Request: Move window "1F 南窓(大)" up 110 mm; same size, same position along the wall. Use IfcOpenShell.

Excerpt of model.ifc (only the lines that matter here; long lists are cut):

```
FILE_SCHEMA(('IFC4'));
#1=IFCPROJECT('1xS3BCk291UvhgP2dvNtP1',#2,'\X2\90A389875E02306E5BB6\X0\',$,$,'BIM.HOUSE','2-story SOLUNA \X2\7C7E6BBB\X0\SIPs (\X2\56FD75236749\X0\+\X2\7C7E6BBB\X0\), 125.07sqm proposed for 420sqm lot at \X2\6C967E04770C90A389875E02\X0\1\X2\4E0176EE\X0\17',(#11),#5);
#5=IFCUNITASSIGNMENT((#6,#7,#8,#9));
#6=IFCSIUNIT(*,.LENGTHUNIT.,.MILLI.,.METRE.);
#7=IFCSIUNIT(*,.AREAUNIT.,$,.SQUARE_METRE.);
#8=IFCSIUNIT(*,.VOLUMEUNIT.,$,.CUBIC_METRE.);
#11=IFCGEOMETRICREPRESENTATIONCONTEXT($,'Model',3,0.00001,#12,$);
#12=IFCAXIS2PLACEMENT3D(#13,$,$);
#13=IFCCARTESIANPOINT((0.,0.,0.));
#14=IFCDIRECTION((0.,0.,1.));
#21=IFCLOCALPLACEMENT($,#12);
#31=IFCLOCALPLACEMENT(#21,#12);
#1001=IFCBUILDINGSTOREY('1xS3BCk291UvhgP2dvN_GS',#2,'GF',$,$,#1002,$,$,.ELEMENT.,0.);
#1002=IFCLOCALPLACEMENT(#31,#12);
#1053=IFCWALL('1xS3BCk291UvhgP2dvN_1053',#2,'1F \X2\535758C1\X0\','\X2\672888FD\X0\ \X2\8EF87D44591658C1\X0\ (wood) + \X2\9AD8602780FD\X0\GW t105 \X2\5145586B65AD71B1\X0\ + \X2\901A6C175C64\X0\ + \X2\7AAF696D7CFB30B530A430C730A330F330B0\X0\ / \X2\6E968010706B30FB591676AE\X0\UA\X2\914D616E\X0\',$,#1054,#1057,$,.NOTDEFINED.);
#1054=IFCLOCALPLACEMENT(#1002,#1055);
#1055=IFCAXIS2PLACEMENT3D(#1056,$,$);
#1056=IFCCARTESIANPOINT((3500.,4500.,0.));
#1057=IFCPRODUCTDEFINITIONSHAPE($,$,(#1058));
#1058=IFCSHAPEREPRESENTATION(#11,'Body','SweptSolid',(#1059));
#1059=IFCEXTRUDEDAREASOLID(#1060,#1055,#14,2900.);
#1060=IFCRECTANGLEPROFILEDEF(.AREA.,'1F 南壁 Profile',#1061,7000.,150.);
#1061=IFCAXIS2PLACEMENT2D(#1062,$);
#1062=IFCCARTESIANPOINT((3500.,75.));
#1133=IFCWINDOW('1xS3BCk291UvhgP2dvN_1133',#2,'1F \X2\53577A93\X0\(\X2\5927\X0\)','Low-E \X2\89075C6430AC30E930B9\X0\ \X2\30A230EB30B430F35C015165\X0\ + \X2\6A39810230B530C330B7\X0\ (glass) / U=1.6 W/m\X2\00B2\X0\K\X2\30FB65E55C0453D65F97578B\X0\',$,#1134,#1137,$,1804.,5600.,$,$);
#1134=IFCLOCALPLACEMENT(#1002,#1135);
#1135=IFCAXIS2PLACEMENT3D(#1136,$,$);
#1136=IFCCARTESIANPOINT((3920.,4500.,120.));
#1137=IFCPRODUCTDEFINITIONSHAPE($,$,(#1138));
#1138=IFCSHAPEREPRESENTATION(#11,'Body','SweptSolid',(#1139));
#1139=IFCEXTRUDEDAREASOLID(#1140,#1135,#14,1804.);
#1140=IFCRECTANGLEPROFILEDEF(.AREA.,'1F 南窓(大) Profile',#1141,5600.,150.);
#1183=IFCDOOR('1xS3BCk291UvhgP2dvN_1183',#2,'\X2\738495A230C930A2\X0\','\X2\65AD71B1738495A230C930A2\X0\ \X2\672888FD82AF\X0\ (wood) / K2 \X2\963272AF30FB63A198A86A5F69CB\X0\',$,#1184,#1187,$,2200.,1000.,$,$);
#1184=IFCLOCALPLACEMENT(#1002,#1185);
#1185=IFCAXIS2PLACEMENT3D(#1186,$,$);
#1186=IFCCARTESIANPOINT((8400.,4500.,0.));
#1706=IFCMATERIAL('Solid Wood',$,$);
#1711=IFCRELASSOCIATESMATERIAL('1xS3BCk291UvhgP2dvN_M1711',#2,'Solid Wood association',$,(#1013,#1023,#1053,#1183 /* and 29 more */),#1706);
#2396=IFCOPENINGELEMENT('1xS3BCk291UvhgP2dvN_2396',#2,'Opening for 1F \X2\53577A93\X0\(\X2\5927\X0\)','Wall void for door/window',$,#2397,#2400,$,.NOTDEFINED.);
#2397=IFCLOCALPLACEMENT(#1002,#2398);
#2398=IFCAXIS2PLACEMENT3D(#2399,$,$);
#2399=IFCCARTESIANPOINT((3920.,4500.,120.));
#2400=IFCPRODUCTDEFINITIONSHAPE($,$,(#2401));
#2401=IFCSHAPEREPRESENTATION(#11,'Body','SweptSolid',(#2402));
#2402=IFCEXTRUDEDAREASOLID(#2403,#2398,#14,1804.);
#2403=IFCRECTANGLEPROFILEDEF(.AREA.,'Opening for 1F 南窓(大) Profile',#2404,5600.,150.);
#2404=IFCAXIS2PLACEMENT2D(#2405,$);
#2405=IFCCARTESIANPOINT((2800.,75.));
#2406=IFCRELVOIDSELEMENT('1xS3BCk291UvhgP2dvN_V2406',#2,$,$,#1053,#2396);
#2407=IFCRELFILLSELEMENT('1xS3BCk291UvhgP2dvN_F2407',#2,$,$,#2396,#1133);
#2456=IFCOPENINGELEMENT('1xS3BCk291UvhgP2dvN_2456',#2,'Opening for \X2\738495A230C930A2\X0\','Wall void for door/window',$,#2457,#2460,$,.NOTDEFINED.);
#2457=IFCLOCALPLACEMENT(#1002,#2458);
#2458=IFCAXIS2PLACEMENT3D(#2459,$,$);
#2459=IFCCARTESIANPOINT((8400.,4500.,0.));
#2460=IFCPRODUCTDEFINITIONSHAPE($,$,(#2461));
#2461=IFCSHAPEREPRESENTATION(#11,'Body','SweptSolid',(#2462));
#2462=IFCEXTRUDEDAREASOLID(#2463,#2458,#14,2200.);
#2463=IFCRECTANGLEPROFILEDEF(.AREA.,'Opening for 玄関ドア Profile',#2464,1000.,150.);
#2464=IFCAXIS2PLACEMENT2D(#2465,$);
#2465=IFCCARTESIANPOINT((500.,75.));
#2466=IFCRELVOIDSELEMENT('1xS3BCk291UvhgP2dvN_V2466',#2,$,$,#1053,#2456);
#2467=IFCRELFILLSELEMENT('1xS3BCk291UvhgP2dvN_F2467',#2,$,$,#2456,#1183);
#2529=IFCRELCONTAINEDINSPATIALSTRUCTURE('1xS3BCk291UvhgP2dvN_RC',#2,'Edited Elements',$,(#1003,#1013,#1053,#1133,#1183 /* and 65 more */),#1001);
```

```python
import numpy as np
import ifcopenshell
import ifcopenshell.api.geometry
import ifcopenshell.util.placement
import ifcopenshell.util.unit

model = ifcopenshell.open("model.ifc")
unit_scale = ifcopenshell.util.unit.calculate_unit_scale(model)

window = model.by_id(1133)
opening = window.FillsVoids[0].RelatingOpeningElement
dz = 110.0

shift = np.array([0.0, 0.0, dz])
# The window is not placed relative to its opening, so move both.
for product in (opening, window):
    matrix = ifcopenshell.util.placement.get_local_placement(product.ObjectPlacement)
    matrix[:3, 3] += shift
    ifcopenshell.api.geometry.edit_object_placement(model, product=product, matrix=matrix, is_si=False)

print(f"moved by {dz * unit_scale:+.3f} m")

model.write("model_edited.ifc")
```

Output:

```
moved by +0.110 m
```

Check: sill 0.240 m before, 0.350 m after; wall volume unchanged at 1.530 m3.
